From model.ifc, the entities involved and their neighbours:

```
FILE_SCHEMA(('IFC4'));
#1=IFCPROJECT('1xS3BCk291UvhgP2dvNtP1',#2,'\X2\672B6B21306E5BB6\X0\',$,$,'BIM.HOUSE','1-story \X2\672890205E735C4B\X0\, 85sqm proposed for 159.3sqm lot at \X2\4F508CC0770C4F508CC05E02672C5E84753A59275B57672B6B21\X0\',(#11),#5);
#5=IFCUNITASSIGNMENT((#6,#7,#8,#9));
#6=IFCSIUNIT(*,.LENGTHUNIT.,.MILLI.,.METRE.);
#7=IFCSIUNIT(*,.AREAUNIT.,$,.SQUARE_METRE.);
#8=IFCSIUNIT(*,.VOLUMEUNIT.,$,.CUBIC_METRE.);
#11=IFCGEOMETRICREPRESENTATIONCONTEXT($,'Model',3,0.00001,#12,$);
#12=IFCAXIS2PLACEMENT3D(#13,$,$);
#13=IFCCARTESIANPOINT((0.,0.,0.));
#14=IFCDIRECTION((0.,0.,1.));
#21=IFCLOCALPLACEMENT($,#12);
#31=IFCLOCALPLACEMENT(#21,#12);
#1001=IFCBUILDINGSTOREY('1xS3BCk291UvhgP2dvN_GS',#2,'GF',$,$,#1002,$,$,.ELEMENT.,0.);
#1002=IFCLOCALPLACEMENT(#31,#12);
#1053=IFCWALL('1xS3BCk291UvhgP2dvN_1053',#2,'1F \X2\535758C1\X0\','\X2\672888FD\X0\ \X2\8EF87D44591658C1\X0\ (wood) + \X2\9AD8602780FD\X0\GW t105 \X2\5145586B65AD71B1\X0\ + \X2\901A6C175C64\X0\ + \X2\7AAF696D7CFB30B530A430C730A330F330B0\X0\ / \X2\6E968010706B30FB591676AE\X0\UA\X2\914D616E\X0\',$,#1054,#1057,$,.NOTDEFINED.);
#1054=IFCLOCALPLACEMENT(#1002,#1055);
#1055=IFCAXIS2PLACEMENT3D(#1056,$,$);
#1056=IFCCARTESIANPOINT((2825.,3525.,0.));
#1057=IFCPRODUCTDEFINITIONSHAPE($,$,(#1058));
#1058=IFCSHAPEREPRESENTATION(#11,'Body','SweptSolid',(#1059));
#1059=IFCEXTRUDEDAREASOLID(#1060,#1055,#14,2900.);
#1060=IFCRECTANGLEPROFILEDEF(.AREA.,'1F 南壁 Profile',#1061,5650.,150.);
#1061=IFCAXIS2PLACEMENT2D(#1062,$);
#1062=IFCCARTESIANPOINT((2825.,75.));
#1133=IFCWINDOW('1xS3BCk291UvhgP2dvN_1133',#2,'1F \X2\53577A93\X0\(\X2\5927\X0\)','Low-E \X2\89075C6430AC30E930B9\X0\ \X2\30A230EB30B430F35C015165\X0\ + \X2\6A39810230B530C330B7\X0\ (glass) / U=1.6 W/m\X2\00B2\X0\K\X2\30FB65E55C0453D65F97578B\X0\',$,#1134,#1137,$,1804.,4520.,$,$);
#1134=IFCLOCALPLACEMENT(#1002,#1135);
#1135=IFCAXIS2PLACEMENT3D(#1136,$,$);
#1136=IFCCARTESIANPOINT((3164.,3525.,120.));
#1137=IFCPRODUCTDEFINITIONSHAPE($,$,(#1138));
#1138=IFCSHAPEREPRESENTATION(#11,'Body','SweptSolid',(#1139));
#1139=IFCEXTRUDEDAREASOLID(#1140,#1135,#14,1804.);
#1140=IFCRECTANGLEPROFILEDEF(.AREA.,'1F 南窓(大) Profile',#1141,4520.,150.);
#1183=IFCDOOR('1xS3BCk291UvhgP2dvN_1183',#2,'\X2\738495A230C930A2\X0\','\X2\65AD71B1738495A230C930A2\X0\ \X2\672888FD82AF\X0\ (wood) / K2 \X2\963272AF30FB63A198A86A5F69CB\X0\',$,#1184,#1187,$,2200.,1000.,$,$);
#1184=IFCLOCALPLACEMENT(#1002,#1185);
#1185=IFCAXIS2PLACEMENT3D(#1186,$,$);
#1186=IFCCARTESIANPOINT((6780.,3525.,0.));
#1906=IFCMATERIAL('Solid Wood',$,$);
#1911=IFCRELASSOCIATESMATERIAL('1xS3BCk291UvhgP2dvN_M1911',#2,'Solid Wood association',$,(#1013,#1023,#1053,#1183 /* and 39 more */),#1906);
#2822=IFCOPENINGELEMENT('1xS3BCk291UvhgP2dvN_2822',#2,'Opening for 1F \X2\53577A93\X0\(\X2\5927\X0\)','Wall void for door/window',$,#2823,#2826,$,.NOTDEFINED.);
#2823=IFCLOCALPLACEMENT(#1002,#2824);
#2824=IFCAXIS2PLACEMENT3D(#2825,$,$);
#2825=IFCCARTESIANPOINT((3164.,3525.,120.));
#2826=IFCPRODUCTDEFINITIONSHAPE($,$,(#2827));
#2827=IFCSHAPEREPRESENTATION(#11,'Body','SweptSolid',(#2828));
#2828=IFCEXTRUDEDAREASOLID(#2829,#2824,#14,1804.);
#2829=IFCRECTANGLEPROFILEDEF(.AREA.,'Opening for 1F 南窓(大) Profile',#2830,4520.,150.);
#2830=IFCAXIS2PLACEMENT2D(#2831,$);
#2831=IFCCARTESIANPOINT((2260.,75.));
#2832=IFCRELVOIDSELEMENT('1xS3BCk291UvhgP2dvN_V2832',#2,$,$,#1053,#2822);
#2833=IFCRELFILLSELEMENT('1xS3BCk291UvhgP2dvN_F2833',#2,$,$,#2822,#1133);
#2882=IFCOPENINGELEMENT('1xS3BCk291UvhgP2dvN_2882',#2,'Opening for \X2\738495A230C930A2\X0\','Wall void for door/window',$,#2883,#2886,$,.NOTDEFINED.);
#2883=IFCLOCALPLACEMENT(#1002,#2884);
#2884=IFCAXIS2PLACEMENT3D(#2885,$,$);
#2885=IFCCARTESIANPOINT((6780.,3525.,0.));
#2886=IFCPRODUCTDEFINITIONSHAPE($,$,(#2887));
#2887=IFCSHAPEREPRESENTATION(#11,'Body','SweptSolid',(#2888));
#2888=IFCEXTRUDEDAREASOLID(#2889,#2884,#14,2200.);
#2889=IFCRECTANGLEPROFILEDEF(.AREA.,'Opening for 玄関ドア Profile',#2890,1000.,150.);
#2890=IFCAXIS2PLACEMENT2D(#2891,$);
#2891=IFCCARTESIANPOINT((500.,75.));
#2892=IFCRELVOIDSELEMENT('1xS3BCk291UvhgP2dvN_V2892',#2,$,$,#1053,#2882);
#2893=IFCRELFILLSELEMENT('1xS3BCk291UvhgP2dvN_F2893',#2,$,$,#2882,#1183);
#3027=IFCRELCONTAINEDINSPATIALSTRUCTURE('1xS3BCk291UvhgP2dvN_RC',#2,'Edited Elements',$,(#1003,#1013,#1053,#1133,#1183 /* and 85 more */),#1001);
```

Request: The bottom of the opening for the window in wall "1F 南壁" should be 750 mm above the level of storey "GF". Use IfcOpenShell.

```python
import numpy as np
import ifcopenshell
import ifcopenshell.api.geometry
import ifcopenshell.geom
import ifcopenshell.util.element
import ifcopenshell.util.placement
import ifcopenshell.util.shape
import ifcopenshell.util.unit

model = ifcopenshell.open("model.ifc")
unit_scale = ifcopenshell.util.unit.calculate_unit_scale(model)

window = model.by_id(1133)
opening = window.FillsVoids[0].RelatingOpeningElement
storey = ifcopenshell.util.element.get_container(window, ifc_class="IfcBuildingStorey")
level = ifcopenshell.util.placement.get_local_placement(storey.ObjectPlacement)[2, 3]

# The opening's origin need not be at the sill, so measure its lowest point.
shape = ifcopenshell.geom.create_shape(ifcopenshell.geom.settings(), opening)
bottom = ifcopenshell.util.shape.get_shape_bottom_elevation(shape, shape.geometry) / unit_scale
dz = level + 750.0 - bottom

shift = np.array([0.0, 0.0, dz])
# The window is not placed relative to its opening, so move both.
for product in (opening, window):
    matrix = ifcopenshell.util.placement.get_local_placement(product.ObjectPlacement)
    matrix[:3, 3] += shift
    ifcopenshell.api.geometry.edit_object_placement(model, product=product, matrix=matrix, is_si=False)

print(f"moved by {dz * unit_scale:+.3f} m")

model.write("model_updated.ifc")
```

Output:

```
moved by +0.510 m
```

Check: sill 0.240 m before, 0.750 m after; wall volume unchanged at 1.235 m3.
